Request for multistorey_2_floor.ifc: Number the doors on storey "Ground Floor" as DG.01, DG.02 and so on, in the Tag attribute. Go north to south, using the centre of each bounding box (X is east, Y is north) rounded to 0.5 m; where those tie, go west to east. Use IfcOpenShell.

First a look at what the model holds.

```python
import ifcopenshell
import ifcopenshell.util.element
import ifcopenshell.util.placement

model = ifcopenshell.open("multistorey_2_floor.ifc")
print(model.schema)
storey = next(s for s in model.by_type("IfcBuildingStorey") if s.Name == "Ground Floor")
doors = [e for e in ifcopenshell.util.element.get_decomposition(storey) if e.is_a("IfcDoor")]
for e in sorted(doors, key=lambda e: e.id()):
    origin = ifcopenshell.util.placement.get_local_placement(e.ObjectPlacement)[:3, 3]
    print(e.id(), e.Tag, e.Name, origin.round(2) + 0.0, sep=" | ")
```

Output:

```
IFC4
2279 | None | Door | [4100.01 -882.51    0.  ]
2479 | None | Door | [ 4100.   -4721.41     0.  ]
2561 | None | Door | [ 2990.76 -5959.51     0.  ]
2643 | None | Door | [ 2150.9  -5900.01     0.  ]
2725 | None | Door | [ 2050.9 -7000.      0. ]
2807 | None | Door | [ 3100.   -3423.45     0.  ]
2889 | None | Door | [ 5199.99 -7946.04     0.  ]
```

```python
import ifcopenshell
import ifcopenshell.geom
import ifcopenshell.util.element
import ifcopenshell.util.shape

model = ifcopenshell.open("multistorey_2_floor.ifc")
settings = ifcopenshell.geom.settings()
settings.set("use-world-coords", True)


def centre(element):
    shape = ifcopenshell.geom.create_shape(settings, element)
    return ifcopenshell.util.shape.get_bbox_centroid(shape.geometry)


storey = next(s for s in model.by_type("IfcBuildingStorey") if s.Name == "Ground Floor")
doors = [e for e in ifcopenshell.util.element.get_decomposition(storey) if e.is_a("IfcDoor")]

# Insertion points can sit at a corner or the storey origin, so sort by the geometry (in metres).
centres = {e: centre(e) for e in doors}
doors.sort(key=lambda e: (-round(centres[e][1] / 0.5), centres[e][0]))

for i, e in enumerate(doors, start=1):
    number = f"DG.{i:02d}"
    e.Tag = number
    print(e.id(), number)

model.write("multistorey_2_floor-out.ifc")
```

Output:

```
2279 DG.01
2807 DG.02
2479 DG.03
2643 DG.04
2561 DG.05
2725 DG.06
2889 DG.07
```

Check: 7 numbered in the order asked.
